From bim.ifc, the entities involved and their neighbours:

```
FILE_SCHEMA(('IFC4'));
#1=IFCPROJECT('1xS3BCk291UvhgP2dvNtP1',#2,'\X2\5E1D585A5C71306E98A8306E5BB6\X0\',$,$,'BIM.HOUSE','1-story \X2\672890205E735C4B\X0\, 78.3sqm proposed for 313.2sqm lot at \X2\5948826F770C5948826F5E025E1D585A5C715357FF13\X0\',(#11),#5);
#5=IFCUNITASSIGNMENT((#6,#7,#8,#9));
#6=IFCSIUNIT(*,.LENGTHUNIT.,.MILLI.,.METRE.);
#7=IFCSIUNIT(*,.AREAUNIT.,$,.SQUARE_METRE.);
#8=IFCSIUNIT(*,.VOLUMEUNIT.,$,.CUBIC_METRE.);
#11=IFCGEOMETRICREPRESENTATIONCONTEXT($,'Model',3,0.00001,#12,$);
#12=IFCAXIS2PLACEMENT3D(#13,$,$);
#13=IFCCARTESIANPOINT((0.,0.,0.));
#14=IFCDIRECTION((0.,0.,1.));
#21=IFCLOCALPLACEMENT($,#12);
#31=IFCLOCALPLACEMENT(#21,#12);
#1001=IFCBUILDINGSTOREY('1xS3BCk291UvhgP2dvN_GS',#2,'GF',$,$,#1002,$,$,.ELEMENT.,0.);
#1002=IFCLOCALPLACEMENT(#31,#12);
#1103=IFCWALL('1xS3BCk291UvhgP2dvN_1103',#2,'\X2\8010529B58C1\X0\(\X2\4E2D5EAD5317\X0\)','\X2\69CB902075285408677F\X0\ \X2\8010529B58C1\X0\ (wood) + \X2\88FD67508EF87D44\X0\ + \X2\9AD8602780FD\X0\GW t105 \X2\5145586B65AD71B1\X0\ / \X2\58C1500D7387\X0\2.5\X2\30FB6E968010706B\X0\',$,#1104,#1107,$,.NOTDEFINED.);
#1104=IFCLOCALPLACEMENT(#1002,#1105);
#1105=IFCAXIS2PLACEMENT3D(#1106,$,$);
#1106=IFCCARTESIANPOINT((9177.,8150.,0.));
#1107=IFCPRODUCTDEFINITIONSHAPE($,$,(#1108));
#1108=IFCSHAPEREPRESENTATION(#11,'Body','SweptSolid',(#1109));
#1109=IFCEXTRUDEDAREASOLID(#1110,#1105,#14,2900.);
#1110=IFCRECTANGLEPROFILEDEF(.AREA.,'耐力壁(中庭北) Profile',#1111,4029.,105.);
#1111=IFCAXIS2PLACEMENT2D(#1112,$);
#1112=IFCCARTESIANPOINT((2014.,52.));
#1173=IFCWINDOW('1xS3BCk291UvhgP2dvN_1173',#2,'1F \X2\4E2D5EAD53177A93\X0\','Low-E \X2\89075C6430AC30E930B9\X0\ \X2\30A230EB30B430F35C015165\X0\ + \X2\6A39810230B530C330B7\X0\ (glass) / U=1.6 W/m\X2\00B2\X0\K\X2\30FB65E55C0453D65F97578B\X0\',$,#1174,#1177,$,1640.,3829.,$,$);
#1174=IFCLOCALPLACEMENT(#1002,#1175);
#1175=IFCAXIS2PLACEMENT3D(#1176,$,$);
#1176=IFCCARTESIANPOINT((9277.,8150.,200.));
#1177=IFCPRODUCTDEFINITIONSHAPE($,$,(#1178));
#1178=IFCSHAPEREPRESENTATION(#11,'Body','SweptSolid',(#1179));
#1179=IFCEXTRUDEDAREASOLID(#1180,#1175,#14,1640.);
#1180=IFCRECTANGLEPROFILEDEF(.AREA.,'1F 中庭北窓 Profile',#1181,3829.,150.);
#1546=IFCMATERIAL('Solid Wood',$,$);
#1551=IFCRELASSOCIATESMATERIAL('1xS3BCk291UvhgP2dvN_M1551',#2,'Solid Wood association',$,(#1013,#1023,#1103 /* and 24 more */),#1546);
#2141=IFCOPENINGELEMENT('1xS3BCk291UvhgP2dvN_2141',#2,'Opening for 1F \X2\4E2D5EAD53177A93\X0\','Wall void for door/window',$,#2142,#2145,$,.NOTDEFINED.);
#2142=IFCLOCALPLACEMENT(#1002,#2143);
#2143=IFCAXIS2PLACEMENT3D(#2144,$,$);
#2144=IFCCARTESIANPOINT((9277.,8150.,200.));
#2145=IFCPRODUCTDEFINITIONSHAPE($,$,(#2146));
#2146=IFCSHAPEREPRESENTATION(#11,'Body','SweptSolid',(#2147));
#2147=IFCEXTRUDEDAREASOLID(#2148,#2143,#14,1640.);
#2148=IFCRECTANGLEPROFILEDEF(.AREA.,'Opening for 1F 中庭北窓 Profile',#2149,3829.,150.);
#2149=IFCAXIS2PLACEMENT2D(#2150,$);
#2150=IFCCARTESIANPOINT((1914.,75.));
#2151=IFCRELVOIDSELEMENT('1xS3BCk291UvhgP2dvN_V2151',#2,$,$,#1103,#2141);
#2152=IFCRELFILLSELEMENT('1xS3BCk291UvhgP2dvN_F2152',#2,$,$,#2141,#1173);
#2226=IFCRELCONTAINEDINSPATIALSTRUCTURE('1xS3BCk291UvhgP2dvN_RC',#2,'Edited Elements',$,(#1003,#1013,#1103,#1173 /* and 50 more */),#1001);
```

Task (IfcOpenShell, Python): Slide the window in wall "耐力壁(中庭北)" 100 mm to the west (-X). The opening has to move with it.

```python
import ifcopenshell
import ifcopenshell.api.geometry
import ifcopenshell.util.placement
import ifcopenshell.util.unit

model = ifcopenshell.open("bim.ifc")
unit_scale = ifcopenshell.util.unit.calculate_unit_scale(model)

window = model.by_id(1173)
opening = window.FillsVoids[0].RelatingOpeningElement
wall = opening.VoidsElements[0].RelatingBuildingElement

wall_matrix = ifcopenshell.util.placement.get_local_placement(wall.ObjectPlacement)
shift = wall_matrix[:3, 0] * -0.1 / unit_scale
before = ifcopenshell.util.placement.get_local_placement(window.ObjectPlacement)[:3, 3].copy()

# The window is not placed relative to its opening, so move both.
for product in (opening, window):
    matrix = ifcopenshell.util.placement.get_local_placement(product.ObjectPlacement)
    matrix[:3, 3] += shift
    ifcopenshell.api.geometry.edit_object_placement(model, product=product, matrix=matrix, is_si=False)

after = ifcopenshell.util.placement.get_local_placement(window.ObjectPlacement)[:3, 3]
print("window moved by", (after - before).round(3) + 0.0)

model.write("bim_v2.ifc")
```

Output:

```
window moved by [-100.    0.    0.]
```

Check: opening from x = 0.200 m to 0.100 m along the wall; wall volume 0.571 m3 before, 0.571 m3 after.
